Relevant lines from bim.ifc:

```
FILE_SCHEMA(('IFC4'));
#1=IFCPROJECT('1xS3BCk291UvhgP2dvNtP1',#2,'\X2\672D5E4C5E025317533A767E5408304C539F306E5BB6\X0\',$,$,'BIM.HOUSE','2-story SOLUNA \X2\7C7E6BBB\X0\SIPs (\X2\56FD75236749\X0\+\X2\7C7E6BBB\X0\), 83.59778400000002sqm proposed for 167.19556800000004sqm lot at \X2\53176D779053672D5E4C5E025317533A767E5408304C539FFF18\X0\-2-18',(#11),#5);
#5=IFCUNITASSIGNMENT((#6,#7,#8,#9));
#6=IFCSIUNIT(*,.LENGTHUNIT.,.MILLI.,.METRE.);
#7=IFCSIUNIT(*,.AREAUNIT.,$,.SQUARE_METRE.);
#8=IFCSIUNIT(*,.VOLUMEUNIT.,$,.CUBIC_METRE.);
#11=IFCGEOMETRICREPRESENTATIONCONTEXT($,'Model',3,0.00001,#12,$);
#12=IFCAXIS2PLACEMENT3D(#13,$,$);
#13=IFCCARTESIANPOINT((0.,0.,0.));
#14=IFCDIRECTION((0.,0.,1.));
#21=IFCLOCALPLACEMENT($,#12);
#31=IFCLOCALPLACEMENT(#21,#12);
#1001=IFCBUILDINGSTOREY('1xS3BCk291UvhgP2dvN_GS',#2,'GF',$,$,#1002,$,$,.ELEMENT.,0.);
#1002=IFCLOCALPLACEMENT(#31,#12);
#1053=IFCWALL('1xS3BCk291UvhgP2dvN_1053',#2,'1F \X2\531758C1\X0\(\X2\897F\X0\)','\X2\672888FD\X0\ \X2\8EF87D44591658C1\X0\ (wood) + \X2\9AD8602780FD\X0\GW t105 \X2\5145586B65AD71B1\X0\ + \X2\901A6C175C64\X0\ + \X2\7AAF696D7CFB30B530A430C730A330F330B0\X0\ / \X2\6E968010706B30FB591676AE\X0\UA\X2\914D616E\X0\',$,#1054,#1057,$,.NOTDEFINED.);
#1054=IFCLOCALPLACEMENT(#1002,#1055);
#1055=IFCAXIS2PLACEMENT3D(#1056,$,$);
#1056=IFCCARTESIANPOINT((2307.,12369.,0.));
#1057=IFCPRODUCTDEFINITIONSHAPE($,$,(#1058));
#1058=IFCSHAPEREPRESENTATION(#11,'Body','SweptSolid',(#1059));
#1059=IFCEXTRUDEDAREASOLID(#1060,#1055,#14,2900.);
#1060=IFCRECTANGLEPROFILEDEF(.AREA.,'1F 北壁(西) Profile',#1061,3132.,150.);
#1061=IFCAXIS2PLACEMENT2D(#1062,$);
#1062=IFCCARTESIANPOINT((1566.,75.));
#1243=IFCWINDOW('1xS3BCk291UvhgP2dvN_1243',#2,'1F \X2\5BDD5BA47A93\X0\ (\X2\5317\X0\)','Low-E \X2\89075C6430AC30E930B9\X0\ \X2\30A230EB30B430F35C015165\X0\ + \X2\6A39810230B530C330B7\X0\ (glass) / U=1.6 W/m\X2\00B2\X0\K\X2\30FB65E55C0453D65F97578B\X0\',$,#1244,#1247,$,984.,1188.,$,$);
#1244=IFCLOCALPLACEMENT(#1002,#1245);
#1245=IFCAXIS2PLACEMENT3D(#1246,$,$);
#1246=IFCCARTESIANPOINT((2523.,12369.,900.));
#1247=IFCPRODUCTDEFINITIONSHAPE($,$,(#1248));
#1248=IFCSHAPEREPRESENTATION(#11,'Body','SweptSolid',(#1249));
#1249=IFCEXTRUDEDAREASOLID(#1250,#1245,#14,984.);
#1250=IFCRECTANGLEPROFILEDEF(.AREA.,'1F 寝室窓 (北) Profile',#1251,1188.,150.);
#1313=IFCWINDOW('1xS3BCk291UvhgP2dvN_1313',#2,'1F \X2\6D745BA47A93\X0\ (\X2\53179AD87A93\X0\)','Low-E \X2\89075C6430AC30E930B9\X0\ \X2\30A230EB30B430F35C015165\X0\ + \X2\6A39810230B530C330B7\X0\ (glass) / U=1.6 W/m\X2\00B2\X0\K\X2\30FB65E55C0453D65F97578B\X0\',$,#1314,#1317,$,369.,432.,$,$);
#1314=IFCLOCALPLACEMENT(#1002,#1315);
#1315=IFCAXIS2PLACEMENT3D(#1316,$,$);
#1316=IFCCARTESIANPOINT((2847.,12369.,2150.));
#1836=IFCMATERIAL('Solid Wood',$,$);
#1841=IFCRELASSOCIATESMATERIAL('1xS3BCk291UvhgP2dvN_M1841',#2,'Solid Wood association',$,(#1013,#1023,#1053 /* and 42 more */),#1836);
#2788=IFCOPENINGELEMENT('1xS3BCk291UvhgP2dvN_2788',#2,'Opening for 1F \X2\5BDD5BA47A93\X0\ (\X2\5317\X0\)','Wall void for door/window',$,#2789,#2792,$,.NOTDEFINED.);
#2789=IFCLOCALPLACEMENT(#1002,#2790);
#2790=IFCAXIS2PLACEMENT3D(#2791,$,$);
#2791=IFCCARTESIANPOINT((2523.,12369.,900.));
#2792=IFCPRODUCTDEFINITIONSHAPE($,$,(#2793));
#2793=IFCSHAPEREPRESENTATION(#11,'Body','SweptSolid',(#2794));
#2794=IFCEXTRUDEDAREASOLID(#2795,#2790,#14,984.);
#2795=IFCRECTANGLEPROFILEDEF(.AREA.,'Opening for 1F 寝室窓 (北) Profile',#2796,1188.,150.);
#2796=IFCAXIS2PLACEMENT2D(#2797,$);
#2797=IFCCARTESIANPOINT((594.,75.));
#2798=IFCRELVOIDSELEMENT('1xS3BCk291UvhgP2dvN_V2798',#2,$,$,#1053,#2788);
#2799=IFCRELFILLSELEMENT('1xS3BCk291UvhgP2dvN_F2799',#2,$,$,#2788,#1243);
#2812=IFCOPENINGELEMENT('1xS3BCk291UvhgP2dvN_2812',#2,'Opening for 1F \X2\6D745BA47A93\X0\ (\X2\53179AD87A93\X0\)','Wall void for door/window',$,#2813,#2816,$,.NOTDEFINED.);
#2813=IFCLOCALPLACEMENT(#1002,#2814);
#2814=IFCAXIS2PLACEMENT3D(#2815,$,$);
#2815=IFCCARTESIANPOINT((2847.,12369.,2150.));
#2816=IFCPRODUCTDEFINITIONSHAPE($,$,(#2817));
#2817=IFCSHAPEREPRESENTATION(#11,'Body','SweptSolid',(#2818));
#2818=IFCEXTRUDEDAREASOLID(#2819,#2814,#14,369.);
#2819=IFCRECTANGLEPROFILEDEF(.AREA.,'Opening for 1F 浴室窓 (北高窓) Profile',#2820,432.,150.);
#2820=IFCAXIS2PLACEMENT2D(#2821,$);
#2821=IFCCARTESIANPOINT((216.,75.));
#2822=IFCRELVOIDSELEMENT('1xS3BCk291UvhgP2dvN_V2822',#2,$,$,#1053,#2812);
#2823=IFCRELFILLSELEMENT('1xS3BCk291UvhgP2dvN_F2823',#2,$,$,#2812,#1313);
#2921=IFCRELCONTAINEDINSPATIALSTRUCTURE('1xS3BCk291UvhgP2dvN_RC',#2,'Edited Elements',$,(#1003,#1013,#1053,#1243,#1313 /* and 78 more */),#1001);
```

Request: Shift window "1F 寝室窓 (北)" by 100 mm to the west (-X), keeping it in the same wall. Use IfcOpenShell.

```python
import ifcopenshell
import ifcopenshell.api.geometry
import ifcopenshell.util.placement
import ifcopenshell.util.unit

model = ifcopenshell.open("bim.ifc")
unit_scale = ifcopenshell.util.unit.calculate_unit_scale(model)

window = model.by_id(1243)
opening = window.FillsVoids[0].RelatingOpeningElement
wall = opening.VoidsElements[0].RelatingBuildingElement

wall_matrix = ifcopenshell.util.placement.get_local_placement(wall.ObjectPlacement)
shift = wall_matrix[:3, 0] * -0.1 / unit_scale
before = ifcopenshell.util.placement.get_local_placement(window.ObjectPlacement)[:3, 3].copy()

# The window is not placed relative to its opening, so move both.
for product in (opening, window):
    matrix = ifcopenshell.util.placement.get_local_placement(product.ObjectPlacement)
    matrix[:3, 3] += shift
    ifcopenshell.api.geometry.edit_object_placement(model, product=product, matrix=matrix, is_si=False)

after = ifcopenshell.util.placement.get_local_placement(window.ObjectPlacement)[:3, 3]
print("window moved by", (after - before).round(3) + 0.0)

model.write("bim_edited.ifc")
```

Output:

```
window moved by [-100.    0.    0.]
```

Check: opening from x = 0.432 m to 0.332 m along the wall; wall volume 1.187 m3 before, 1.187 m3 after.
